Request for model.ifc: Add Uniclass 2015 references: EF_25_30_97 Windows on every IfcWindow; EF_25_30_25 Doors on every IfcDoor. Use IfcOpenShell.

First a look at what the model holds.

```python
import ifcopenshell

model = ifcopenshell.open("model.ifc")
print(model.schema)
print("classifications:", [c.Name for c in model.by_type("IfcClassification")])
for ifc_class in ("IfcDoor", "IfcRoof", "IfcStair", "IfcWall", "IfcWindow"):
    print(ifc_class, len(model.by_type(ifc_class)))
```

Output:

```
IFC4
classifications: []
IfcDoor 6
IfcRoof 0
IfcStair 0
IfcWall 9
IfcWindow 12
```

```python
import ifcopenshell
import ifcopenshell.api.classification

model = ifcopenshell.open("model.ifc")

system = ifcopenshell.api.classification.add_classification(model, classification="Uniclass 2015")

codes = {
    "IfcWindow": ("EF_25_30_97", "Windows"),
    "IfcDoor": ("EF_25_30_25", "Doors"),
}
for ifc_class, (code, name) in codes.items():
    products = model.by_type(ifc_class)
    ifcopenshell.api.classification.add_reference(
        model, products=products, classification=system, identification=code, name=name
    )
    print(code, len(products))

model.write("model_rev.ifc")
```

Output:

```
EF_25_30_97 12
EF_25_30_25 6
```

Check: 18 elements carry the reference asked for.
